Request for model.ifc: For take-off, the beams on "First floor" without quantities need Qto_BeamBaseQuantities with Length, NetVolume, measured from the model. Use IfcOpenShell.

First a look at what the model holds.

```python
import ifcopenshell
import ifcopenshell.util.element
import ifcopenshell.util.unit

model = ifcopenshell.open("model.ifc")
print(model.schema)
for unit_type in ("LENGTHUNIT", "AREAUNIT", "VOLUMEUNIT"):
    print(unit_type, ifcopenshell.util.unit.calculate_unit_scale(model, unit_type))
storey = next(s for s in model.by_type("IfcBuildingStorey") if s.Name == "First floor")
beams = [e for e in ifcopenshell.util.element.get_decomposition(storey) if e.is_a("IfcBeam")]
for e in sorted(beams, key=lambda e: e.id()):
    print(e.id(), e.is_a(), e.Name, list(ifcopenshell.util.element.get_psets(e, qtos_only=True)), sep=" | ")
```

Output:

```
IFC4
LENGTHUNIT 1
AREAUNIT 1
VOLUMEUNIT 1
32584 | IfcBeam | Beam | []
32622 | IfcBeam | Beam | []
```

```python
import ifcopenshell
import ifcopenshell.api.pset
import ifcopenshell.geom
import ifcopenshell.util.element
import ifcopenshell.util.shape
import ifcopenshell.util.unit

model = ifcopenshell.open("model.ifc")
unit_scale = ifcopenshell.util.unit.calculate_unit_scale(model)
volume_scale = ifcopenshell.util.unit.calculate_unit_scale(model, "VOLUMEUNIT")
settings = ifcopenshell.geom.settings()

storey = next(s for s in model.by_type("IfcBuildingStorey") if s.Name == "First floor")
beams = [e for e in ifcopenshell.util.element.get_decomposition(storey) if e.is_a("IfcBeam")]

for e in sorted(beams, key=lambda e: e.id()):
    if ifcopenshell.util.element.get_psets(e, qtos_only=True, should_inherit=False):
        continue
    # Geometry comes back in metres, in the element's own axes.
    shape = ifcopenshell.geom.create_shape(settings, e)
    values = {
        "Length": ifcopenshell.util.shape.get_max_xyz(shape.geometry) / unit_scale,
        "NetVolume": ifcopenshell.util.shape.get_volume(shape.geometry) / volume_scale,
    }
    qto = ifcopenshell.api.pset.add_qto(model, product=e, name="Qto_BeamBaseQuantities")
    ifcopenshell.api.pset.edit_qto(model, qto=qto, properties=values)
    print(e.id(), {k: round(v, 3) for k, v in values.items()})

model.write("model_v2.ifc")
```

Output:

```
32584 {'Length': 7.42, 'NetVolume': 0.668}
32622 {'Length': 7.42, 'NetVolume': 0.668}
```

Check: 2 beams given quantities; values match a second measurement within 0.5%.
